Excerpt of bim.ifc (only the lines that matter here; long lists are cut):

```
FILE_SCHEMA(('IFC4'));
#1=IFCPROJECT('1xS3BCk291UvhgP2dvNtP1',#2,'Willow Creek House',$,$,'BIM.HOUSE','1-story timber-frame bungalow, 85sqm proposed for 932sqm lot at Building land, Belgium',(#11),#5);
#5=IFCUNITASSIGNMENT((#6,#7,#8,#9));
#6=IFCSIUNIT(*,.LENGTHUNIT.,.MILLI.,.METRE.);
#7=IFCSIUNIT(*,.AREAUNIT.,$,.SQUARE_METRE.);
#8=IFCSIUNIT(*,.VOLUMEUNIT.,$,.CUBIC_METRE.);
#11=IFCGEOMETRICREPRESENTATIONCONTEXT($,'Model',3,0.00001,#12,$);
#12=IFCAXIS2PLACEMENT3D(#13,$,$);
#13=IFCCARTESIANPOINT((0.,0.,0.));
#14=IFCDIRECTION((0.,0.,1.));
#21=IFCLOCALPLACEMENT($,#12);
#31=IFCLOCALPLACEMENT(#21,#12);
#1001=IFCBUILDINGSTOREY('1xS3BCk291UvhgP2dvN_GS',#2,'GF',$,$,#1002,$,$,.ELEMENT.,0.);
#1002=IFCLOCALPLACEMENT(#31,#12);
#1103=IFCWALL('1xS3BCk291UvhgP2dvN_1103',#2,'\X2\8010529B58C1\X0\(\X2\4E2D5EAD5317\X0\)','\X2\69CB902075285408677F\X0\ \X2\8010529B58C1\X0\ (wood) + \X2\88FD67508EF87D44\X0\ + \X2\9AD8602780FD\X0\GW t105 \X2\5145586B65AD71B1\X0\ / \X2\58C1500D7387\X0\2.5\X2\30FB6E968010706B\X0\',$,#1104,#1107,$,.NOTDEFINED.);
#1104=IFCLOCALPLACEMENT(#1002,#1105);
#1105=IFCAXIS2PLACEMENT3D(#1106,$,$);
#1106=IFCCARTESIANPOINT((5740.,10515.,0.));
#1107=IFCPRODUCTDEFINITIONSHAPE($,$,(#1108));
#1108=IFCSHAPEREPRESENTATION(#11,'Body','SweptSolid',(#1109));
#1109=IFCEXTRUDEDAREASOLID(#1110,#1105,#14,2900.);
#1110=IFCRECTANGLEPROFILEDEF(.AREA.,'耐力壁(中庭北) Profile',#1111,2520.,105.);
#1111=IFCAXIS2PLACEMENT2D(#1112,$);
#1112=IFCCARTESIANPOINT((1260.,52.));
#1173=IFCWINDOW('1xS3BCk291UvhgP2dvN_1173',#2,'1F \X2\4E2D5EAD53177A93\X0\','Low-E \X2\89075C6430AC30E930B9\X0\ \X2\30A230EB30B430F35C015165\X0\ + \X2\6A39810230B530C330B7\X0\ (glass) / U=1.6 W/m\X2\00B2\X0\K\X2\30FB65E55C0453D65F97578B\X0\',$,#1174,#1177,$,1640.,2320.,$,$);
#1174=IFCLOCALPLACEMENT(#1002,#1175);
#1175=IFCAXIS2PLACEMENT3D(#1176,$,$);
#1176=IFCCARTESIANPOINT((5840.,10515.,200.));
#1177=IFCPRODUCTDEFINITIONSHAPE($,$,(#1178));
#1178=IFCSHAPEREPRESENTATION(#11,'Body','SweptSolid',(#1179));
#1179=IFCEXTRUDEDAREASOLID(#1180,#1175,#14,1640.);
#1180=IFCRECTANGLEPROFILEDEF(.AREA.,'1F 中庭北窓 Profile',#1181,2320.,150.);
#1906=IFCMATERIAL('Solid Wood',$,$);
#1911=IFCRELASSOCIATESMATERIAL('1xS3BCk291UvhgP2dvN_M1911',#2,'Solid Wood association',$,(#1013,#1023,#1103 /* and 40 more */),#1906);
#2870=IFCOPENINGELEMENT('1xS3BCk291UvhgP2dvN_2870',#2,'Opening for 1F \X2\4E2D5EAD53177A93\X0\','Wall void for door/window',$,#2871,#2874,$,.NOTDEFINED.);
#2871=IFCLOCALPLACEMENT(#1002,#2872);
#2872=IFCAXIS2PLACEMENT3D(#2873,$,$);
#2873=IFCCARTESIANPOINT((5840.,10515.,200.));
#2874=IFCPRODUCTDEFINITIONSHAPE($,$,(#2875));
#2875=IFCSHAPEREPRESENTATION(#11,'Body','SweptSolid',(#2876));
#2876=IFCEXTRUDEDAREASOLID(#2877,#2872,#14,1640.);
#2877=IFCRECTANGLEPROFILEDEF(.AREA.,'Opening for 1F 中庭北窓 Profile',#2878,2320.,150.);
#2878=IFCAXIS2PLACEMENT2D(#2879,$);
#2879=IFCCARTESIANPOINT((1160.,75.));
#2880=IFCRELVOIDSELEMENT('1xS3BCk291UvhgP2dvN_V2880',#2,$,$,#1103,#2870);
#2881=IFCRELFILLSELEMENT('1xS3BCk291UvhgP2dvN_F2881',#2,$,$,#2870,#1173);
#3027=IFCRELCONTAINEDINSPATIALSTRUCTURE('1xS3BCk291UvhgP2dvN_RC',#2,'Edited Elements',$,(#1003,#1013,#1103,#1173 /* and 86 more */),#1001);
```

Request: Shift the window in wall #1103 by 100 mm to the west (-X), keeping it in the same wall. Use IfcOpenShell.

```python
import ifcopenshell
import ifcopenshell.api.geometry
import ifcopenshell.util.placement

model = ifcopenshell.open("bim.ifc")

window = model.by_guid("1xS3BCk291UvhgP2dvN_1173")
opening = window.FillsVoids[0].RelatingOpeningElement
wall = opening.VoidsElements[0].RelatingBuildingElement

wall_matrix = ifcopenshell.util.placement.get_local_placement(wall.ObjectPlacement)
shift = wall_matrix[:3, 0] * -100.0
before = ifcopenshell.util.placement.get_local_placement(window.ObjectPlacement)[:3, 3].copy()

# The window is not placed relative to its opening, so move both.
for product in (opening, window):
    matrix = ifcopenshell.util.placement.get_local_placement(product.ObjectPlacement)
    matrix[:3, 3] += shift
    ifcopenshell.api.geometry.edit_object_placement(model, product=product, matrix=matrix, is_si=False)

after = ifcopenshell.util.placement.get_local_placement(window.ObjectPlacement)[:3, 3]
print("window moved by", (after - before).round(3) + 0.0)

model.write("bim_edited.ifc")
```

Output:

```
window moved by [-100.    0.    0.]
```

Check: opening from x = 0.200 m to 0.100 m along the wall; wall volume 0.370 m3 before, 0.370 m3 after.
